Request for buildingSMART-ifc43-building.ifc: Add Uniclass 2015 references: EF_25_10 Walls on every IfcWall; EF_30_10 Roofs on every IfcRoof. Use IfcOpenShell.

First a look at what the model holds.

```python
import ifcopenshell

model = ifcopenshell.open("buildingSMART-ifc43-building.ifc")
print(model.schema)
print("classifications:", [c.Name for c in model.by_type("IfcClassification")])
for ifc_class in ("IfcDoor", "IfcRoof", "IfcStair", "IfcWall", "IfcWindow"):
    print(ifc_class, len(model.by_type(ifc_class)))
```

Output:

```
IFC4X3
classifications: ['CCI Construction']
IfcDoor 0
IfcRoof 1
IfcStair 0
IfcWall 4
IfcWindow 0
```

```python
import ifcopenshell
import ifcopenshell.api.classification

model = ifcopenshell.open("buildingSMART-ifc43-building.ifc")

system = ifcopenshell.api.classification.add_classification(model, classification="Uniclass 2015")

codes = {
    "IfcWall": ("EF_25_10", "Walls"),
    "IfcRoof": ("EF_30_10", "Roofs"),
}
for ifc_class, (code, name) in codes.items():
    products = model.by_type(ifc_class)
    ifcopenshell.api.classification.add_reference(
        model, products=products, classification=system, identification=code, name=name
    )
    print(code, len(products))

model.write("buildingSMART-ifc43-building_rev.ifc")
```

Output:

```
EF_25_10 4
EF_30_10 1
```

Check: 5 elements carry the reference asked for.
